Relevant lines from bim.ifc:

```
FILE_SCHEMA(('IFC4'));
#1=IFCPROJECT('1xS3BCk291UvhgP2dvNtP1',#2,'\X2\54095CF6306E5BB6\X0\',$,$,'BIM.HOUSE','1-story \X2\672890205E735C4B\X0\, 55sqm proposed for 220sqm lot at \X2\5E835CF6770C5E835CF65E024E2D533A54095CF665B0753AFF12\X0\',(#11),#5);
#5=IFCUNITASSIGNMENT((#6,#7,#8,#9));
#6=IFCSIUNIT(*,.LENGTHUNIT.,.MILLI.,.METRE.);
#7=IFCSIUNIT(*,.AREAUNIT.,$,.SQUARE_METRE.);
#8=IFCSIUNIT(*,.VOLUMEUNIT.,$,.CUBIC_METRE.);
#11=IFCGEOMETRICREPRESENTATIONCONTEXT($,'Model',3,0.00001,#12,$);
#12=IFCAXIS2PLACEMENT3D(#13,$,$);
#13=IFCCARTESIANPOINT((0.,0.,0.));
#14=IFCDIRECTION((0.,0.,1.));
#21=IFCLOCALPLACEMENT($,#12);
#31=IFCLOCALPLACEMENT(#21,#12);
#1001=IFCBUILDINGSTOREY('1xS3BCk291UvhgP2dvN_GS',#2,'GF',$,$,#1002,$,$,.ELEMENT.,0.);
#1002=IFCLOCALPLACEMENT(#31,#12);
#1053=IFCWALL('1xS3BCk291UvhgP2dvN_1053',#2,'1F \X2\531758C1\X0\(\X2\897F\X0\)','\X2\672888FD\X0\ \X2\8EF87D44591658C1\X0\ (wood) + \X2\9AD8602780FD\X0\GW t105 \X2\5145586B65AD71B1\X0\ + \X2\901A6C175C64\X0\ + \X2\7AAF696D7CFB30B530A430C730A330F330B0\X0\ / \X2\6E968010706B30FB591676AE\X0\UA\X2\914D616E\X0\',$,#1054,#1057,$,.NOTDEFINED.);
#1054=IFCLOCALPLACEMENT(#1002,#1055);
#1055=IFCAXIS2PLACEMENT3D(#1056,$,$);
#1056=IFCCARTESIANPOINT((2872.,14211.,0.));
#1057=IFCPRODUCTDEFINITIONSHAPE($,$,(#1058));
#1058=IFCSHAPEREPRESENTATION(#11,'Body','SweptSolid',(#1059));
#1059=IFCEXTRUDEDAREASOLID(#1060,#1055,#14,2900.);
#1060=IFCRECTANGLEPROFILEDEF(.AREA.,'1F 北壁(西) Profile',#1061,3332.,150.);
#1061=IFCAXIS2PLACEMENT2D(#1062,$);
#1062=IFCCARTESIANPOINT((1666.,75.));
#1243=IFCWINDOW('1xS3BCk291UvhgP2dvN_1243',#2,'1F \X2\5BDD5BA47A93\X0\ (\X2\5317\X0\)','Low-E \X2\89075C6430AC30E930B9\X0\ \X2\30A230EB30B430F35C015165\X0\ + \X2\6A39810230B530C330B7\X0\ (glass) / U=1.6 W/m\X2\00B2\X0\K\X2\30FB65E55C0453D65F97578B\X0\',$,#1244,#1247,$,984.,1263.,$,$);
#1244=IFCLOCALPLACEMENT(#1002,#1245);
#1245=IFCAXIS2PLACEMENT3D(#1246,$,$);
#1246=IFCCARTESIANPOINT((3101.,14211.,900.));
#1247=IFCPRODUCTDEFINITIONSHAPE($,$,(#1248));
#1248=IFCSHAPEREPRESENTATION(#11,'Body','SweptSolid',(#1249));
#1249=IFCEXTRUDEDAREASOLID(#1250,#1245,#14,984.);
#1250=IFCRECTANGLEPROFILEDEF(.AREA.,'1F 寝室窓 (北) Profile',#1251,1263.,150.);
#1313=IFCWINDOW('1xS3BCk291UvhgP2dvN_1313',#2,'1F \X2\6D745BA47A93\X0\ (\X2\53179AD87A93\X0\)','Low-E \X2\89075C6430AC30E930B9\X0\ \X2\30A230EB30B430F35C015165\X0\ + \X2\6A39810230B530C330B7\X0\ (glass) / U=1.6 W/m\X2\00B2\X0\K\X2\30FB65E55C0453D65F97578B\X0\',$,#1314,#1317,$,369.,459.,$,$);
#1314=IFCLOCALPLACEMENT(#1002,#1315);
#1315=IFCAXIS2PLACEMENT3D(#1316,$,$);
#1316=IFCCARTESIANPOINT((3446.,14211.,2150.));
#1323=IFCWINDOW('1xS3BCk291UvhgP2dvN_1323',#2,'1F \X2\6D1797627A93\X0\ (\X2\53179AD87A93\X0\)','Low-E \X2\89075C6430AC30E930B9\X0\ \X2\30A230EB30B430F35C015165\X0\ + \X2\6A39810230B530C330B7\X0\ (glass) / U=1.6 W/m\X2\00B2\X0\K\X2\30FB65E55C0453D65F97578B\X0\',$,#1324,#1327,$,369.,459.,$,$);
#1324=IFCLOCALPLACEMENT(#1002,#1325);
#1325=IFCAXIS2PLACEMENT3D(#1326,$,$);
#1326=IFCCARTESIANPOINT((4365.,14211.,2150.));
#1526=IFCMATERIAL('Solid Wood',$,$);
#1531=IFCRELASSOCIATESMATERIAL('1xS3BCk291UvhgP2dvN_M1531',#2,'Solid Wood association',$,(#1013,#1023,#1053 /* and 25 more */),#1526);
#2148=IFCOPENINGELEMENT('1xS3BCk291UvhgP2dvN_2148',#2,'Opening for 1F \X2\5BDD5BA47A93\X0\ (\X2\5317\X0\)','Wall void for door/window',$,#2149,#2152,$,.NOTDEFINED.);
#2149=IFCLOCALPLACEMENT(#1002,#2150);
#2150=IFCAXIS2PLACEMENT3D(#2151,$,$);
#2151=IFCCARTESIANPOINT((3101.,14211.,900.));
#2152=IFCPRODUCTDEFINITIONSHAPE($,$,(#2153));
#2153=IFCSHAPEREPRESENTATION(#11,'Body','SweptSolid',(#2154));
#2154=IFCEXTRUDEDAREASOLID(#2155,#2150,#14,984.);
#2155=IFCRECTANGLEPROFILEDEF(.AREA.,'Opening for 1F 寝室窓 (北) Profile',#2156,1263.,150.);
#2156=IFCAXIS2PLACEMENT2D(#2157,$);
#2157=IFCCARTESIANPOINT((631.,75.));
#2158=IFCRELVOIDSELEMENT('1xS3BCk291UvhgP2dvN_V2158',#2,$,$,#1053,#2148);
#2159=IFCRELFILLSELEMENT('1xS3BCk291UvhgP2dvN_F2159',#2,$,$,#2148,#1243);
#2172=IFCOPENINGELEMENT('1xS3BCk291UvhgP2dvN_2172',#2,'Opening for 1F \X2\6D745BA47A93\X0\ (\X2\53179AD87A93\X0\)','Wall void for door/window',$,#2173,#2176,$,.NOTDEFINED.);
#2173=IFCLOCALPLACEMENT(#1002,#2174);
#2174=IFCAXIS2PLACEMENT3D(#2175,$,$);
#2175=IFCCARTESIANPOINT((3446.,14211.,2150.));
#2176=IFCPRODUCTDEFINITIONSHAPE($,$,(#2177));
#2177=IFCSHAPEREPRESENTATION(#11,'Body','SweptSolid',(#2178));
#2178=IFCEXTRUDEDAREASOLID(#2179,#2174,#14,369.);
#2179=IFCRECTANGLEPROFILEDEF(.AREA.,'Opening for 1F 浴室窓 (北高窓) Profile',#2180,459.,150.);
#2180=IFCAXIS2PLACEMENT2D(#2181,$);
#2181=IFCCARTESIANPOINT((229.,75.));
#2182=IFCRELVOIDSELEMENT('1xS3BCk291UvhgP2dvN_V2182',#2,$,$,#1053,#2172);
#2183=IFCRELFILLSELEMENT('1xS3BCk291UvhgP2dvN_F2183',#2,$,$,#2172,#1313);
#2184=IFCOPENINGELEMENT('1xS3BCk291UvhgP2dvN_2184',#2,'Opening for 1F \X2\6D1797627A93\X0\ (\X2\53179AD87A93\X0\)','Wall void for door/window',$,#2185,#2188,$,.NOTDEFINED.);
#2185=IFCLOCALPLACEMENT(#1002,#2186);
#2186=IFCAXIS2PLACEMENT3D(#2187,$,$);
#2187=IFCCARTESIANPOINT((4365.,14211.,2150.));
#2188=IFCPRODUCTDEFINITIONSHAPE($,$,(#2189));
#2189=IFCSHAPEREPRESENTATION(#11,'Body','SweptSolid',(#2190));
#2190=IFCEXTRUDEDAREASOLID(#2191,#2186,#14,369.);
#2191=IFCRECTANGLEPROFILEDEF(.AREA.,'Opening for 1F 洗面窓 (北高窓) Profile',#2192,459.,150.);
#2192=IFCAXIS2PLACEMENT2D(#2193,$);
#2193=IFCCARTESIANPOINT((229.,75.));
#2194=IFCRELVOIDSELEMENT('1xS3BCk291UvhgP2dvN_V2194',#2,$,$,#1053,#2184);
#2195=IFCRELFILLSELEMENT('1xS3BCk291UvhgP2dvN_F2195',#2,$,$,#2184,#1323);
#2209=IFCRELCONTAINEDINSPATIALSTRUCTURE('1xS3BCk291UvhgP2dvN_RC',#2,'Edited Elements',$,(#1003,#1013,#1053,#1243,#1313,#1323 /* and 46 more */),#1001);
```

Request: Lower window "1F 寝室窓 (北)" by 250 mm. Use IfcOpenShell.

```python
import numpy as np
import ifcopenshell
import ifcopenshell.api.geometry
import ifcopenshell.util.placement
import ifcopenshell.util.unit

model = ifcopenshell.open("bim.ifc")
unit_scale = ifcopenshell.util.unit.calculate_unit_scale(model)

window = model.by_guid("1xS3BCk291UvhgP2dvN_1243")
opening = window.FillsVoids[0].RelatingOpeningElement
dz = -250.0

shift = np.array([0.0, 0.0, dz])
# The window is not placed relative to its opening, so move both.
for product in (opening, window):
    matrix = ifcopenshell.util.placement.get_local_placement(product.ObjectPlacement)
    matrix[:3, 3] += shift
    ifcopenshell.api.geometry.edit_object_placement(model, product=product, matrix=matrix, is_si=False)

print(f"moved by {dz * unit_scale:+.3f} m")

model.write("bim-out.ifc")
```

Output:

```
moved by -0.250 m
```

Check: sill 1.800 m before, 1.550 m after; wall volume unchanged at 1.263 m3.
